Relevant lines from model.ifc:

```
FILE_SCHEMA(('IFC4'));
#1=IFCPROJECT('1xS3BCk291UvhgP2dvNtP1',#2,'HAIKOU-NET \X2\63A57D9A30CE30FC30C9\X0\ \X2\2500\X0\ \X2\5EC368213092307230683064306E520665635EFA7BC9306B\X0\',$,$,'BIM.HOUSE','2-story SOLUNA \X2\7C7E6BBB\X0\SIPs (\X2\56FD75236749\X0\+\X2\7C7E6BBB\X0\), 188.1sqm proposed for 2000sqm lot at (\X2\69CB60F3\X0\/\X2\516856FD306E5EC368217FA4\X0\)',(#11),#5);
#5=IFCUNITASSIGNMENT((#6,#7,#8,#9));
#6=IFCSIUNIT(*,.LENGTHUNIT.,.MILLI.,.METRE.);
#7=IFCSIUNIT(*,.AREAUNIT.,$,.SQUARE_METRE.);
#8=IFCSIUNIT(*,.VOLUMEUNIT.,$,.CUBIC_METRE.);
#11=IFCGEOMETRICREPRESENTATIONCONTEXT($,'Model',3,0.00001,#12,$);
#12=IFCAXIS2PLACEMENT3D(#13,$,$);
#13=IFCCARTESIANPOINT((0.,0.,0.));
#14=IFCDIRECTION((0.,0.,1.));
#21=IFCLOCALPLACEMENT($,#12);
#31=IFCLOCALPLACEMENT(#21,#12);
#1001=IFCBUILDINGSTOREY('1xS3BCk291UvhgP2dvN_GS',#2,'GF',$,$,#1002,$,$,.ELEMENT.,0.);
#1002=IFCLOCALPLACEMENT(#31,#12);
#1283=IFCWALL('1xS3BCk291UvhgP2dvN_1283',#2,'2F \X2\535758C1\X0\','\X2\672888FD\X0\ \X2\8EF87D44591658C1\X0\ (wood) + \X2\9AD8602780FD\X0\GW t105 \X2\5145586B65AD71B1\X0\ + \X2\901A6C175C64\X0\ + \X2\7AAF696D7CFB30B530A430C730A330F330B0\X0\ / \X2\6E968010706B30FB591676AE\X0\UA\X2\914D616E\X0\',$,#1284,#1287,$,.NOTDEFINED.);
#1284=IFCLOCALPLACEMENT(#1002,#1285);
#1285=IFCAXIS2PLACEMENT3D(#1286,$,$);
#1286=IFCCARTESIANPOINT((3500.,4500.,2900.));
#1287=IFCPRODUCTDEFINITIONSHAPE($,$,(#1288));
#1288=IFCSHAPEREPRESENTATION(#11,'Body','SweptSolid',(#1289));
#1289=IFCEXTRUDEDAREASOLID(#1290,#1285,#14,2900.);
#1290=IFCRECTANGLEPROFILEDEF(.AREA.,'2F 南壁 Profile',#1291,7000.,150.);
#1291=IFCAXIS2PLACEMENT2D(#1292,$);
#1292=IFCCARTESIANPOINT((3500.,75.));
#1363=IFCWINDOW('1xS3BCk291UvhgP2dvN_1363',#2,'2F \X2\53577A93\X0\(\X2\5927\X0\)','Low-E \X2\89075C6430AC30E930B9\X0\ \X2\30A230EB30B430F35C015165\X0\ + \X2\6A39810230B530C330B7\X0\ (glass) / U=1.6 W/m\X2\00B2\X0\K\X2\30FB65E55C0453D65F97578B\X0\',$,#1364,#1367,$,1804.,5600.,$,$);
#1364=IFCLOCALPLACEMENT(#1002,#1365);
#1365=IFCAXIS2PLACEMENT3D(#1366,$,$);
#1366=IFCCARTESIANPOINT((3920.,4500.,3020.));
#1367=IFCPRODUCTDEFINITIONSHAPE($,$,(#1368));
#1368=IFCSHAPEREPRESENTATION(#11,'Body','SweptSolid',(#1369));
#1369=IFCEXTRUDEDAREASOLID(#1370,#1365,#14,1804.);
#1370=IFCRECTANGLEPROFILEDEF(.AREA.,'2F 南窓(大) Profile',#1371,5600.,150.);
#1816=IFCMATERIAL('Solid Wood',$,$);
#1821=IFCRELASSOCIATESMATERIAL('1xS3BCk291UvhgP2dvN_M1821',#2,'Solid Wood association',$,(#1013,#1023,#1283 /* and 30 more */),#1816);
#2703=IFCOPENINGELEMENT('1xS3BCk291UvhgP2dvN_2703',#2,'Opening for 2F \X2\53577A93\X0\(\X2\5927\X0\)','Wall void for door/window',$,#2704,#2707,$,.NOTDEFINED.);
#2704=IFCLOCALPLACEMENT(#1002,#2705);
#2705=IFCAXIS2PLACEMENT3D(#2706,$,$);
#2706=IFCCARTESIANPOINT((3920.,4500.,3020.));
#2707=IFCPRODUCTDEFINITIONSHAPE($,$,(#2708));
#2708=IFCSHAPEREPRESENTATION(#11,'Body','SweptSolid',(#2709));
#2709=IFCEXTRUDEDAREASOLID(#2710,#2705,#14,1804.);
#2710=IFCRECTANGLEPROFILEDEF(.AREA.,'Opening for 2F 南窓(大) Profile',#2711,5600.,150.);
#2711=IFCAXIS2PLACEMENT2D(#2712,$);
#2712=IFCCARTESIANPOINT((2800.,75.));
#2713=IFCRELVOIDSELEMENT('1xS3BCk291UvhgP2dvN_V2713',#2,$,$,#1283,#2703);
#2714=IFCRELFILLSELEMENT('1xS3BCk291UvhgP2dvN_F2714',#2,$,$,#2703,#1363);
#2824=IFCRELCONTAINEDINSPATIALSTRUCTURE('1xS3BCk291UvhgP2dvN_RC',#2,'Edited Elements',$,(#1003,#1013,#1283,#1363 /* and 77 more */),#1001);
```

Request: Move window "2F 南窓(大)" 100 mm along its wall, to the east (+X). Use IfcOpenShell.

```python
import ifcopenshell
import ifcopenshell.api.geometry
import ifcopenshell.util.placement

model = ifcopenshell.open("model.ifc")

window = model.by_guid("1xS3BCk291UvhgP2dvN_1363")
opening = window.FillsVoids[0].RelatingOpeningElement
wall = opening.VoidsElements[0].RelatingBuildingElement

wall_matrix = ifcopenshell.util.placement.get_local_placement(wall.ObjectPlacement)
shift = wall_matrix[:3, 0] * 100.0
before = ifcopenshell.util.placement.get_local_placement(window.ObjectPlacement)[:3, 3].copy()

# The window is not placed relative to its opening, so move both.
for product in (opening, window):
    matrix = ifcopenshell.util.placement.get_local_placement(product.ObjectPlacement)
    matrix[:3, 3] += shift
    ifcopenshell.api.geometry.edit_object_placement(model, product=product, matrix=matrix, is_si=False)

after = ifcopenshell.util.placement.get_local_placement(window.ObjectPlacement)[:3, 3]
print("window moved by", (after - before).round(3) + 0.0)

model.write("model-out.ifc")
```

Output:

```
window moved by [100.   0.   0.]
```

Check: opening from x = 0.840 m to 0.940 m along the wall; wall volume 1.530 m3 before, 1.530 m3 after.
